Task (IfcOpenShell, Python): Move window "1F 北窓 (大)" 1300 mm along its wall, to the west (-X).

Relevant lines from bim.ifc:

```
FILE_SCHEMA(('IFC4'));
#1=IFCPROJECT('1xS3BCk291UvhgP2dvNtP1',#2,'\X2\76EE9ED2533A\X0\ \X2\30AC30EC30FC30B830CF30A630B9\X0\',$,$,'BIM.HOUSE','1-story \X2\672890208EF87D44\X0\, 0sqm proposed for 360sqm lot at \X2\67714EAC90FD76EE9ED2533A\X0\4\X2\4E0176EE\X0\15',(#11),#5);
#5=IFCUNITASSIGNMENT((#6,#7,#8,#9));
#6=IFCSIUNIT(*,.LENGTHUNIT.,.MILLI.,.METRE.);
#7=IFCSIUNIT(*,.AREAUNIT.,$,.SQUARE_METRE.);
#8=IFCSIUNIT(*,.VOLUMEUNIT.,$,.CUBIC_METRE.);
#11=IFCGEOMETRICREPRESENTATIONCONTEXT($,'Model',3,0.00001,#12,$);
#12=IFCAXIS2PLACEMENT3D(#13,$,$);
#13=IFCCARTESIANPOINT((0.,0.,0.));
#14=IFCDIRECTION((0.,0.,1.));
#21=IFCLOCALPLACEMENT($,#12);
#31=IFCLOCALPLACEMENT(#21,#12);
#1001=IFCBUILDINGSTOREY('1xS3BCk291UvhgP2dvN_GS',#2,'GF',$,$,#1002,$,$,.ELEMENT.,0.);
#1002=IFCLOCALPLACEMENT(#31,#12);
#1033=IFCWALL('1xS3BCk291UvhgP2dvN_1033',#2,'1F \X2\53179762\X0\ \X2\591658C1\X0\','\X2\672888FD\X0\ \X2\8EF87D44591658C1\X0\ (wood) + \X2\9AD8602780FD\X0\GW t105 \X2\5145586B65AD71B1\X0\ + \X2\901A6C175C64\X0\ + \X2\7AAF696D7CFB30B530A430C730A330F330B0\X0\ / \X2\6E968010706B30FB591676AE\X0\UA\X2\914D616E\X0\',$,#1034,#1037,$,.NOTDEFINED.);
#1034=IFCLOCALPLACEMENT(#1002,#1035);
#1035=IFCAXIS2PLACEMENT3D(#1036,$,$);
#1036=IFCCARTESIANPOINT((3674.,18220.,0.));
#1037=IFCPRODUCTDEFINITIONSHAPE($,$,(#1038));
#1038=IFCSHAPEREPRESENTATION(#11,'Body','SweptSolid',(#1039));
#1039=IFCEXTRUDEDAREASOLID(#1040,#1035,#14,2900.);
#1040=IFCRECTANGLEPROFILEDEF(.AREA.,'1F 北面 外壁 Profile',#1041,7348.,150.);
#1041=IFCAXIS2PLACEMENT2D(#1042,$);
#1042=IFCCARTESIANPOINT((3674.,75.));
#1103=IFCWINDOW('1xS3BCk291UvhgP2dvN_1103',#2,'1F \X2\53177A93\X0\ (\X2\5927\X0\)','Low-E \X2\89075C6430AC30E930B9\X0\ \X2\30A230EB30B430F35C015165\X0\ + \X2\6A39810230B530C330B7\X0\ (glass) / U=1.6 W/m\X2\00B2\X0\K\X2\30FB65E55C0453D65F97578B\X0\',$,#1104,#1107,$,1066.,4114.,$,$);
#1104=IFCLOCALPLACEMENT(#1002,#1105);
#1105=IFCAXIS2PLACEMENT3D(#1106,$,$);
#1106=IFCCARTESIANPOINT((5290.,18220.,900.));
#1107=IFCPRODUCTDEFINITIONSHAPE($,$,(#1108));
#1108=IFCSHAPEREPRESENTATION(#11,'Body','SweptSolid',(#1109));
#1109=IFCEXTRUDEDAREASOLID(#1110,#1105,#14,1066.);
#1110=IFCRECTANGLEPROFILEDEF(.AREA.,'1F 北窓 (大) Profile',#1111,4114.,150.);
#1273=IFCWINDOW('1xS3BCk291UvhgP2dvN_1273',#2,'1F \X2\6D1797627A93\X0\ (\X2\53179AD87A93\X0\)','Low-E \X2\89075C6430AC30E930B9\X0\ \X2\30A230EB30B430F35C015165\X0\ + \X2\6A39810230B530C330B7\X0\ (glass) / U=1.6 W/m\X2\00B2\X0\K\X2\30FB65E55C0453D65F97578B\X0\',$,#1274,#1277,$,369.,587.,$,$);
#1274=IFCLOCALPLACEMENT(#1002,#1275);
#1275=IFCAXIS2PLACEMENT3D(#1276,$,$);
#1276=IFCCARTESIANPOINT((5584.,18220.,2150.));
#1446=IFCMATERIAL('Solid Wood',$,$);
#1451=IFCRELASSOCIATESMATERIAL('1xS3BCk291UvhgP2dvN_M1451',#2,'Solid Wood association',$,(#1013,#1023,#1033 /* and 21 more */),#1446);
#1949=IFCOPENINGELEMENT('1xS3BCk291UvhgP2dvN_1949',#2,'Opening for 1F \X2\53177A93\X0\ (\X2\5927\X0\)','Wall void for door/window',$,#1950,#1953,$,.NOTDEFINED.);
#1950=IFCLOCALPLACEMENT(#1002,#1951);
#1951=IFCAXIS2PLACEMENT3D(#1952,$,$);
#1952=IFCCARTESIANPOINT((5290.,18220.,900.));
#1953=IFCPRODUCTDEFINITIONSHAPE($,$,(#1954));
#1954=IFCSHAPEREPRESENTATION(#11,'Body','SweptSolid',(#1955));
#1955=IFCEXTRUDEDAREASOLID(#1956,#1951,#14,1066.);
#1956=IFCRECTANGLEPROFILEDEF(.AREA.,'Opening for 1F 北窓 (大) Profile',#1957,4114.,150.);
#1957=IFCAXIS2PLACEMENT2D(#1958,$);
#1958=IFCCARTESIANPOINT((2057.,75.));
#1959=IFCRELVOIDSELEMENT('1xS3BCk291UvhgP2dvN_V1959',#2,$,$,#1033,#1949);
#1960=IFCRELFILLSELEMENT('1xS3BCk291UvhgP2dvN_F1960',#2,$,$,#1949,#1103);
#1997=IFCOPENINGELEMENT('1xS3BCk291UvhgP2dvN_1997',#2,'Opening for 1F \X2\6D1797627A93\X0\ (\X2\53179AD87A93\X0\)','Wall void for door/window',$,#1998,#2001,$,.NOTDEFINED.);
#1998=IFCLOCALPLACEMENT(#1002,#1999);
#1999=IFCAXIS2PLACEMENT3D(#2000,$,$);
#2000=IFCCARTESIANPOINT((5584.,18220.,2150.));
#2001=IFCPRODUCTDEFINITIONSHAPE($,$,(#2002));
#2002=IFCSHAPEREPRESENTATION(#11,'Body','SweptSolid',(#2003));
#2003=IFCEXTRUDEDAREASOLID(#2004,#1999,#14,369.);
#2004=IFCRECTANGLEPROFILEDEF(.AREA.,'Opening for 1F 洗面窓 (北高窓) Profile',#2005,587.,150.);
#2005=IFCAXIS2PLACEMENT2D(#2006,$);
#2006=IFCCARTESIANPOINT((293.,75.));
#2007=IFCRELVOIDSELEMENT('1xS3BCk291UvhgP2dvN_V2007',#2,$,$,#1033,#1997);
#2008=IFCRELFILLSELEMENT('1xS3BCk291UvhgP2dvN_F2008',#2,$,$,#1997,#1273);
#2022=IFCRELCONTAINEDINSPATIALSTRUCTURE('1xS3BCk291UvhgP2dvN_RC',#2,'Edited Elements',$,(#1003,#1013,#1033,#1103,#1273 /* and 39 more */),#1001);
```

```python
import ifcopenshell
import ifcopenshell.api.geometry
import ifcopenshell.util.placement

model = ifcopenshell.open("bim.ifc")

window = model.by_guid("1xS3BCk291UvhgP2dvN_1103")
opening = window.FillsVoids[0].RelatingOpeningElement
wall = opening.VoidsElements[0].RelatingBuildingElement

wall_matrix = ifcopenshell.util.placement.get_local_placement(wall.ObjectPlacement)
shift = wall_matrix[:3, 0] * -1300.0
before = ifcopenshell.util.placement.get_local_placement(window.ObjectPlacement)[:3, 3].copy()

# The window is not placed relative to its opening, so move both.
for product in (opening, window):
    matrix = ifcopenshell.util.placement.get_local_placement(product.ObjectPlacement)
    matrix[:3, 3] += shift
    ifcopenshell.api.geometry.edit_object_placement(model, product=product, matrix=matrix, is_si=False)

after = ifcopenshell.util.placement.get_local_placement(window.ObjectPlacement)[:3, 3]
print("window moved by", (after - before).round(3) + 0.0)

model.write("bim_v2.ifc")
```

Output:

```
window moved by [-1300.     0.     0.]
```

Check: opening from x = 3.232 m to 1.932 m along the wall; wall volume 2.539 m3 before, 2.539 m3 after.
